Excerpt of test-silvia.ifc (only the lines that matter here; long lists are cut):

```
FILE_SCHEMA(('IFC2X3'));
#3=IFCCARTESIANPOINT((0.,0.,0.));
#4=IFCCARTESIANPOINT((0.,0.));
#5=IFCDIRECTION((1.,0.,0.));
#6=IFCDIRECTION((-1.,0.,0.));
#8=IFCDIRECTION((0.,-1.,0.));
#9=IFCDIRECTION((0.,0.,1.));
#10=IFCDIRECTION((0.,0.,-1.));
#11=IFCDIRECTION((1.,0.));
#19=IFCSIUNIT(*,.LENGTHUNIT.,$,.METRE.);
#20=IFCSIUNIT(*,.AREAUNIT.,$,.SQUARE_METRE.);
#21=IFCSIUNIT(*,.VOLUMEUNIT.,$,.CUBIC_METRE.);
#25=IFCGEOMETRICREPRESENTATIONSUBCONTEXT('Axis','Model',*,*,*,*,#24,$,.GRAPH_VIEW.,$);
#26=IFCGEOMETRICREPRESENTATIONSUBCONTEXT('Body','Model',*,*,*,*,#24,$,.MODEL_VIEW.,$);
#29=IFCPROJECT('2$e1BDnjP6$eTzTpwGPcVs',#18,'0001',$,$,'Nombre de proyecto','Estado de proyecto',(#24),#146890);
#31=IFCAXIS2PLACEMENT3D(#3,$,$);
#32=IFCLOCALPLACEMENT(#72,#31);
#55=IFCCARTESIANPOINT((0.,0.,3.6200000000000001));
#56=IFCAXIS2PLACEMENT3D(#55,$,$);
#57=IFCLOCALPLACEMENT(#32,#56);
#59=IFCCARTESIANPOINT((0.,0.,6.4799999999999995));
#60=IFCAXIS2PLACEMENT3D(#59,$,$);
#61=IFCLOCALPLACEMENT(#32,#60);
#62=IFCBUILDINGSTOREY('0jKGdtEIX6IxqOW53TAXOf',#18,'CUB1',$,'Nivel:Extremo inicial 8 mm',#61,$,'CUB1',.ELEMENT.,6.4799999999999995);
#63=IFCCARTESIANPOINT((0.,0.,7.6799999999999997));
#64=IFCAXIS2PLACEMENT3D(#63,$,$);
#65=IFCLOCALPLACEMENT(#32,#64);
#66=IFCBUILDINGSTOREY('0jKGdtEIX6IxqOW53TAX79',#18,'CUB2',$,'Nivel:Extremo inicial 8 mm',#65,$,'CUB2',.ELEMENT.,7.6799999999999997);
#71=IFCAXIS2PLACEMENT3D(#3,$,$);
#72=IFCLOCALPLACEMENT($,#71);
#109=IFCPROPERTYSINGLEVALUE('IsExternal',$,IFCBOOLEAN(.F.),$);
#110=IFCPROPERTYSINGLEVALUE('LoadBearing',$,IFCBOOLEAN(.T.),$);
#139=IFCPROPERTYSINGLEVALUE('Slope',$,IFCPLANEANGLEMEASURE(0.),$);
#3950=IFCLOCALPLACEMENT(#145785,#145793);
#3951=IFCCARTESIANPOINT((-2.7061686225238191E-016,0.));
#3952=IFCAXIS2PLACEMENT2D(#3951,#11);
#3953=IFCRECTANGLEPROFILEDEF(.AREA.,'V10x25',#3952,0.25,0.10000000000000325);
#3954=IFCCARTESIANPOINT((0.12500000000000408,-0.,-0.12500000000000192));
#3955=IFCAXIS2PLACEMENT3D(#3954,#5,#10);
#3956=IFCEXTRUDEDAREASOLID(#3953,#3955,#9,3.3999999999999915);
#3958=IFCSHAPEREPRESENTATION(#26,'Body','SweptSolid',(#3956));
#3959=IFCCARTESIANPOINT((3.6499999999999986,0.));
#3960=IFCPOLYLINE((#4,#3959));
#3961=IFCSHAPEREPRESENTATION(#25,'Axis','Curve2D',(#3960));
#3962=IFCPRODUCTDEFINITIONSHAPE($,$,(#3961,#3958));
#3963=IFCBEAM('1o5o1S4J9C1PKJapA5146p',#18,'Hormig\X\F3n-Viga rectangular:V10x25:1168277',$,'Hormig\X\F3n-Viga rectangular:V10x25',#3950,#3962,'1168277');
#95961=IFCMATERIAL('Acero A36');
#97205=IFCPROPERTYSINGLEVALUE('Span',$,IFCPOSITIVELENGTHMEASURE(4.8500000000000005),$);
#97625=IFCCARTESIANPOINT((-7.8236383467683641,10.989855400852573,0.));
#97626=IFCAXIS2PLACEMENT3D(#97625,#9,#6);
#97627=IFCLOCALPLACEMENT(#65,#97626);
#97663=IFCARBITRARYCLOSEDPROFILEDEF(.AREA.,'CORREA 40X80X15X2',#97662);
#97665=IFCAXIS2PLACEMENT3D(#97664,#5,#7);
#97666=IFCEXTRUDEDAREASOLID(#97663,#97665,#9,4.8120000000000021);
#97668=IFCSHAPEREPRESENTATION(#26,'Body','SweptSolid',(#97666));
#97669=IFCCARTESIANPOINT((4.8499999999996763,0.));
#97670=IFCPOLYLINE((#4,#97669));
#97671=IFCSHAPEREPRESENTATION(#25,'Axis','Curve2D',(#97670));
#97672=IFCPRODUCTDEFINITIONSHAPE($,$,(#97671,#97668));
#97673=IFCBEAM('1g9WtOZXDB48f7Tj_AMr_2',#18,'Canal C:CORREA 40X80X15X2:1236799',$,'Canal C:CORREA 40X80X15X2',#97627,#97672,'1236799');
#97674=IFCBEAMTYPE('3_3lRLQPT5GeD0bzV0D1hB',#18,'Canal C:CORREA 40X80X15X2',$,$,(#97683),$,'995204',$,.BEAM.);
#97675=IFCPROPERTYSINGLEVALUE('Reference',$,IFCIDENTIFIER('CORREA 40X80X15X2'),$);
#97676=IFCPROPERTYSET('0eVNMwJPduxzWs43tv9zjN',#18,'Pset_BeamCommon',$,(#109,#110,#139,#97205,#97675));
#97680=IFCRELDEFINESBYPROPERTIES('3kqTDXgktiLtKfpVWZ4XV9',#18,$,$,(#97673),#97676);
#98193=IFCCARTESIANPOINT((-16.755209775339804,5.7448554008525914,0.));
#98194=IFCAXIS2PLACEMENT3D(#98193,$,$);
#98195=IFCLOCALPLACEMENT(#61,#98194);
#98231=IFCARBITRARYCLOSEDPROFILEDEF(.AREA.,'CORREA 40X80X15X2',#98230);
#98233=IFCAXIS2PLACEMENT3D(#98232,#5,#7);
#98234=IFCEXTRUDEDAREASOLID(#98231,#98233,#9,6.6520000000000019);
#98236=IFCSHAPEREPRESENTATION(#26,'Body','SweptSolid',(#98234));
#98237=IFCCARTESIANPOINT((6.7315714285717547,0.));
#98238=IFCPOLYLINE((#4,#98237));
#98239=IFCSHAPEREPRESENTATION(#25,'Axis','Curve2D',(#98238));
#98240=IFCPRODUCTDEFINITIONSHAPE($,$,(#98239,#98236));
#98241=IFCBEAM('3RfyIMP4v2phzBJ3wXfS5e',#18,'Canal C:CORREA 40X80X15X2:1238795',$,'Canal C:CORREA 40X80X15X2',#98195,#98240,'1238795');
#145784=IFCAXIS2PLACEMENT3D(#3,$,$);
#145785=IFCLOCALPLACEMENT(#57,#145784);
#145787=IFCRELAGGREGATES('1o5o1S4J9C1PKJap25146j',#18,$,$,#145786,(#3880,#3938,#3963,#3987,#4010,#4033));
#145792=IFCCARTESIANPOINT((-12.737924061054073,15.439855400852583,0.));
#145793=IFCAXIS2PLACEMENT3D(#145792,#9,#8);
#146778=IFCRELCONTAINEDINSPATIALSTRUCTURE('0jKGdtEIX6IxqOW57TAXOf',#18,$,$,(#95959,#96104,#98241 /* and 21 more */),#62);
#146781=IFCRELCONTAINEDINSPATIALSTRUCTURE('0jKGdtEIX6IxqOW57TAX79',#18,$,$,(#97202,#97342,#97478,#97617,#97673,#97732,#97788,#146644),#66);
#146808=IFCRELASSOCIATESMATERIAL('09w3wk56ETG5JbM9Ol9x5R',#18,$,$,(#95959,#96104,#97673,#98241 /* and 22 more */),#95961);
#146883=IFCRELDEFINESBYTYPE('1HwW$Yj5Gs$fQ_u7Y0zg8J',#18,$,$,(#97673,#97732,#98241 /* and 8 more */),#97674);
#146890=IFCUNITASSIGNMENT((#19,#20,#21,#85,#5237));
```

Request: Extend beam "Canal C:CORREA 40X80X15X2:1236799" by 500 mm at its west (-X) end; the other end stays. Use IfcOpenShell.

```python
import numpy as np
import ifcopenshell
import ifcopenshell.api.pset
import ifcopenshell.util.element
import ifcopenshell.util.representation

model = ifcopenshell.open("test-silvia.ifc")

member = model.by_guid("1g9WtOZXDB48f7Tj_AMr_2")
change = 0.5

# The extrusion runs towards the end named, so only its depth changes.
body = ifcopenshell.util.representation.get_representation(member, "Model", "Body")
solid = body.Items[0]
old_length = solid.Depth
solid.Depth += change

# Move the axis end point with it.
axis = next(r for r in member.Representation.Representations if r.RepresentationIdentifier == "Axis").Items[0]
start, end = (np.array(p.Coordinates) for p in axis.Points)
end = end + (end - start) / np.linalg.norm(end - start) * change
point = model.createIfcCartesianPoint(end.tolist())
axis.Points = [axis.Points[0], point]

# Update the stored length and volume.
pset = model.by_id(ifcopenshell.util.element.get_pset(member, "Pset_BeamCommon", should_inherit=False)["id"])
ifcopenshell.api.pset.edit_pset(model, pset=pset, properties={
    "Span": model.create_entity("IfcPositiveLengthMeasure", solid.Depth),
})

print(f"length {old_length:g} -> {solid.Depth:g}")

model.write("test-silvia_rev.ifc")
```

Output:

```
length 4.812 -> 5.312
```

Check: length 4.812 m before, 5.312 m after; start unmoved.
